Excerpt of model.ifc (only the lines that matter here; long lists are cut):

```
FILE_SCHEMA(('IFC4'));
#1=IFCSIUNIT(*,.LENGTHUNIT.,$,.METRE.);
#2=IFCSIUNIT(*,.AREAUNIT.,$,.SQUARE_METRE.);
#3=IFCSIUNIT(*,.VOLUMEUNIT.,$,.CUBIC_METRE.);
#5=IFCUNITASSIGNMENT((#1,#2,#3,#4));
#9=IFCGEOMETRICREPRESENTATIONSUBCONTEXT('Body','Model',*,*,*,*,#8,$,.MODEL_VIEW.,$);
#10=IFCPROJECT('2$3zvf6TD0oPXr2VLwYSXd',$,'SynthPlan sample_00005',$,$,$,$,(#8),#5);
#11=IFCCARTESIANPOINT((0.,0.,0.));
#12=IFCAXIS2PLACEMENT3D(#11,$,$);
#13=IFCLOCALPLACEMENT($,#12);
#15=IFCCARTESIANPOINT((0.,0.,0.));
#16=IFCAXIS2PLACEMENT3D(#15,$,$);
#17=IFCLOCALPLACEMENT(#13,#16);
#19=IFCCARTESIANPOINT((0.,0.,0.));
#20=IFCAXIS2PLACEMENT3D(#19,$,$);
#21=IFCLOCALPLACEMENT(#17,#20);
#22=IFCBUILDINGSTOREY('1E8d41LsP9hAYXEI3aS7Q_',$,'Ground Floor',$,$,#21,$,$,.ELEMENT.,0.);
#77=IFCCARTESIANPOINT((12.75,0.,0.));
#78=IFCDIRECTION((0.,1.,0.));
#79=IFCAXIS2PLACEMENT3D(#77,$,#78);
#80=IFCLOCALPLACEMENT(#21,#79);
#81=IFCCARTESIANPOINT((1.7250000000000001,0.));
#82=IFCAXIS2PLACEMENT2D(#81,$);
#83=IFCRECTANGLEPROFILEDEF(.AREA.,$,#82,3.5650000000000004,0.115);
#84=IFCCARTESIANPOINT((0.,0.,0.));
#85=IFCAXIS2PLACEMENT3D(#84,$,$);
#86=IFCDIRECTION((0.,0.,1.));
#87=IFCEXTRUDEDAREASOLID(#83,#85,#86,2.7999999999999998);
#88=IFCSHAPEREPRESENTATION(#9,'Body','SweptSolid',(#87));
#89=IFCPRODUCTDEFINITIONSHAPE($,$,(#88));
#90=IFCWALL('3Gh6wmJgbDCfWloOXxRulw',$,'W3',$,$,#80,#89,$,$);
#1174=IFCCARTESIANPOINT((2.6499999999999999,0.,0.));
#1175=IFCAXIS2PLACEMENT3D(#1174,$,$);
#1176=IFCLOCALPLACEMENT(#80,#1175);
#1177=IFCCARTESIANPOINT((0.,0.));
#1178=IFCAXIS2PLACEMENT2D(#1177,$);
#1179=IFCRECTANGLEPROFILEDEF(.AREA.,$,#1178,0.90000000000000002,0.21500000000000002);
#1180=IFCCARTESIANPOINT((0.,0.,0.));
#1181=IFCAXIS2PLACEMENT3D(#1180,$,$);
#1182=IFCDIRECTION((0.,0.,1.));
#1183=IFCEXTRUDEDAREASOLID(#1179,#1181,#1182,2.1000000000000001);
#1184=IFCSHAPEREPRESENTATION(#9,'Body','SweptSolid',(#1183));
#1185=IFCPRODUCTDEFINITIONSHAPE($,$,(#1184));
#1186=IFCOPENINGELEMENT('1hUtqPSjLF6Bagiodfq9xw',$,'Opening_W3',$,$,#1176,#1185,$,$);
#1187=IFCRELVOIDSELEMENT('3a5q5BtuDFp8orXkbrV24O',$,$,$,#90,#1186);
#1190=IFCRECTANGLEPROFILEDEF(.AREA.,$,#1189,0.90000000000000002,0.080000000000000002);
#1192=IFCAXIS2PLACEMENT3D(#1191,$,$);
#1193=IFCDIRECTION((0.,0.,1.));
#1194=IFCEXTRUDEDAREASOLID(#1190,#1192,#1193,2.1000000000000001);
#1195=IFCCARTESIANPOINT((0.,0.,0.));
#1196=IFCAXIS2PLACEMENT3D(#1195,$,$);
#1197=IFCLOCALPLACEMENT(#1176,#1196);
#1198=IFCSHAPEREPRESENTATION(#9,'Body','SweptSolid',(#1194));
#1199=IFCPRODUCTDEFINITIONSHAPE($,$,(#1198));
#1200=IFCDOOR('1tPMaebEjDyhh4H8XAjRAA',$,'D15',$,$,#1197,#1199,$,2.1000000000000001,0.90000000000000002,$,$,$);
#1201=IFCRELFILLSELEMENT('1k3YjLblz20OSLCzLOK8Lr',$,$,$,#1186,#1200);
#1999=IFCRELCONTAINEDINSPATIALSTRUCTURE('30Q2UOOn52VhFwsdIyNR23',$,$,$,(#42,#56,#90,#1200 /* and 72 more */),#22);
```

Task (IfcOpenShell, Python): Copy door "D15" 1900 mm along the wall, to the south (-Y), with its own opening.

```python
import ifcopenshell
import ifcopenshell.api.feature
import ifcopenshell.api.geometry
import ifcopenshell.api.root
import ifcopenshell.geom
import ifcopenshell.util.element
import ifcopenshell.util.placement
import ifcopenshell.util.shape

model = ifcopenshell.open("model.ifc")
settings = ifcopenshell.geom.settings()


def volume(element):
    """Net volume in cubic metres, openings subtracted."""
    shape = ifcopenshell.geom.create_shape(settings, element)
    return ifcopenshell.util.shape.get_volume(shape.geometry)


door = model.by_guid("1tPMaebEjDyhh4H8XAjRAA")
opening = door.FillsVoids[0].RelatingOpeningElement
wall = opening.VoidsElements[0].RelatingBuildingElement
before = volume(wall)
shift = ifcopenshell.util.placement.get_local_placement(wall.ObjectPlacement)[:3, 0] * -1.9

# copy_class copies the void relationship, type, container and properties, but no geometry.
new_opening = ifcopenshell.api.root.copy_class(model, product=opening)
new_opening.Representation = ifcopenshell.util.element.copy_deep(
    model, opening.Representation, exclude=["IfcGeometricRepresentationContext", "IfcRepresentationMap"]
)
new_door = ifcopenshell.api.root.copy_class(model, product=door)
new_door.Representation = ifcopenshell.util.element.copy_deep(
    model, door.Representation, exclude=["IfcGeometricRepresentationContext", "IfcRepresentationMap"]
)
ifcopenshell.api.feature.add_filling(model, opening=new_opening, element=new_door)

for old, new in ((opening, new_opening), (door, new_door)):
    matrix = ifcopenshell.util.placement.get_local_placement(old.ObjectPlacement)
    matrix[:3, 3] += shift
    ifcopenshell.api.geometry.edit_object_placement(model, product=new, matrix=matrix, is_si=False)

after = volume(wall)

print(f"wall volume {before:.3f} -> {after:.3f} m3")

model.write("model_edited.ifc")
```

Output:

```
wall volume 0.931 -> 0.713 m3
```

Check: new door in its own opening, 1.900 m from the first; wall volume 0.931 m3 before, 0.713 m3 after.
